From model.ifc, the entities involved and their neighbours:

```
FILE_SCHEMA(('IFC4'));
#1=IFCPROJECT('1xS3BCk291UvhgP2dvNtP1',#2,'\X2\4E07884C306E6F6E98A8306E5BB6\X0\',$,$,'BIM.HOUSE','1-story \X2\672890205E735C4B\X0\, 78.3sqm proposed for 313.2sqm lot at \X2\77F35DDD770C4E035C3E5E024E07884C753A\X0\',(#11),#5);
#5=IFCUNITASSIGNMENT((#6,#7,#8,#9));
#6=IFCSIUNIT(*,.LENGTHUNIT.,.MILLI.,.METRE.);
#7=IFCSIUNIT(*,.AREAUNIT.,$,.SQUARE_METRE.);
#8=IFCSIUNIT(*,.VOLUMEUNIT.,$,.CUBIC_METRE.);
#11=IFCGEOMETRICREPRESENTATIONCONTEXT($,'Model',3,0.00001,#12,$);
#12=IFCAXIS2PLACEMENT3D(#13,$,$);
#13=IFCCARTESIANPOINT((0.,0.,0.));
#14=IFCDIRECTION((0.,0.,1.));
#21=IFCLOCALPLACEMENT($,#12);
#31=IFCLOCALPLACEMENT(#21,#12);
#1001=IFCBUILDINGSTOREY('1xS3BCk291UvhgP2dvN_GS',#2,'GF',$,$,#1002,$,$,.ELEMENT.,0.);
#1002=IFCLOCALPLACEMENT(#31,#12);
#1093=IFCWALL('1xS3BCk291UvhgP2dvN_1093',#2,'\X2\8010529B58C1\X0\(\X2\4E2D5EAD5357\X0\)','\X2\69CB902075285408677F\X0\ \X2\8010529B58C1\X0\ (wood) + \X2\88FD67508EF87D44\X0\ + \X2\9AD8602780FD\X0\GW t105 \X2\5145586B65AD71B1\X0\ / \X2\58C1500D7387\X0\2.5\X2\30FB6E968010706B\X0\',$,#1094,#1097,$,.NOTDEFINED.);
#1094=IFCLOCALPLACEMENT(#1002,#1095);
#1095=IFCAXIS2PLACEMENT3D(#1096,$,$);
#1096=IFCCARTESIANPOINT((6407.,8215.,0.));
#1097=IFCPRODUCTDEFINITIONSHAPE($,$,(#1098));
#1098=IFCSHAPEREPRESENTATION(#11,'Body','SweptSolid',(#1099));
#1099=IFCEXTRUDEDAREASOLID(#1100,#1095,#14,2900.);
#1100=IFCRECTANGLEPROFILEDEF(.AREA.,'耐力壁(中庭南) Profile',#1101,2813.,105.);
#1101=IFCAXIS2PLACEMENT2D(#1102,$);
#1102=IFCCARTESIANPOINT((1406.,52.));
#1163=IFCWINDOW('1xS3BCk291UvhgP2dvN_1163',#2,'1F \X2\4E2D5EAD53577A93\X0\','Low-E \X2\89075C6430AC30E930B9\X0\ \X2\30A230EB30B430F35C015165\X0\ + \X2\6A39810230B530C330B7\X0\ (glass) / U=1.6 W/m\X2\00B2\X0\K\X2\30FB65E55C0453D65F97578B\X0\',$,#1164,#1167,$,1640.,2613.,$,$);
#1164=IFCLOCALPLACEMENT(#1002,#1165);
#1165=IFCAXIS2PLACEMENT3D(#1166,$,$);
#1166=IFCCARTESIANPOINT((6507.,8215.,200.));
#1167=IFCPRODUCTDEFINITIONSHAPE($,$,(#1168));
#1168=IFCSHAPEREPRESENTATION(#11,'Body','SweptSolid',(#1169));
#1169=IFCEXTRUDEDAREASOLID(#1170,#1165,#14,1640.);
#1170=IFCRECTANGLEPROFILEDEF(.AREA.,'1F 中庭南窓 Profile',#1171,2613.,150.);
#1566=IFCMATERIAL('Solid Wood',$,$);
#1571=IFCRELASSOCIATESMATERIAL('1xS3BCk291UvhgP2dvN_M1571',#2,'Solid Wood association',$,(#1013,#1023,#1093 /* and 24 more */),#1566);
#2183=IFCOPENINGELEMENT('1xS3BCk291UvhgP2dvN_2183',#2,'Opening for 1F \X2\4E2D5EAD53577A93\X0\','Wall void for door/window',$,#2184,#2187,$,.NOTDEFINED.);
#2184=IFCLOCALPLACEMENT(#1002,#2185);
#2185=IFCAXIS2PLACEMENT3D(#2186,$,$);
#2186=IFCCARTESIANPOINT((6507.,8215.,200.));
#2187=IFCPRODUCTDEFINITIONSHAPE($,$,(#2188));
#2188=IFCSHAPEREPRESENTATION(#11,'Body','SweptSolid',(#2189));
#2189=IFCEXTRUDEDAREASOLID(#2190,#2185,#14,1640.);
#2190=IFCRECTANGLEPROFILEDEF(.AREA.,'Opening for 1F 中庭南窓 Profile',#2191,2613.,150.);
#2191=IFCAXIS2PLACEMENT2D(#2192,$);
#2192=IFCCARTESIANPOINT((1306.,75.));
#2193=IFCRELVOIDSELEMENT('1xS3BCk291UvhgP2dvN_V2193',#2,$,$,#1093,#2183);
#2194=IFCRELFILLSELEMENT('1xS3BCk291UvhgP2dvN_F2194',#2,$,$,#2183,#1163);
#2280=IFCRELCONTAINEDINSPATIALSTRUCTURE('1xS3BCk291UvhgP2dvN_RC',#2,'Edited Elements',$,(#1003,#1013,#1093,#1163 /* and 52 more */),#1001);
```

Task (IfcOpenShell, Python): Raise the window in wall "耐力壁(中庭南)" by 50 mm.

```python
import numpy as np
import ifcopenshell
import ifcopenshell.api.geometry
import ifcopenshell.util.placement
import ifcopenshell.util.unit

model = ifcopenshell.open("model.ifc")
unit_scale = ifcopenshell.util.unit.calculate_unit_scale(model)

window = model.by_guid("1xS3BCk291UvhgP2dvN_1163")
opening = window.FillsVoids[0].RelatingOpeningElement
dz = 0.05 / unit_scale

shift = np.array([0.0, 0.0, dz])
# The window is not placed relative to its opening, so move both.
for product in (opening, window):
    matrix = ifcopenshell.util.placement.get_local_placement(product.ObjectPlacement)
    matrix[:3, 3] += shift
    ifcopenshell.api.geometry.edit_object_placement(model, product=product, matrix=matrix, is_si=False)

print(f"moved by {dz * unit_scale:+.3f} m")

model.write("model_rev.ifc")
```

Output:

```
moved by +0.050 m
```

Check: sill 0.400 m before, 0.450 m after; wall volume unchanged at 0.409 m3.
